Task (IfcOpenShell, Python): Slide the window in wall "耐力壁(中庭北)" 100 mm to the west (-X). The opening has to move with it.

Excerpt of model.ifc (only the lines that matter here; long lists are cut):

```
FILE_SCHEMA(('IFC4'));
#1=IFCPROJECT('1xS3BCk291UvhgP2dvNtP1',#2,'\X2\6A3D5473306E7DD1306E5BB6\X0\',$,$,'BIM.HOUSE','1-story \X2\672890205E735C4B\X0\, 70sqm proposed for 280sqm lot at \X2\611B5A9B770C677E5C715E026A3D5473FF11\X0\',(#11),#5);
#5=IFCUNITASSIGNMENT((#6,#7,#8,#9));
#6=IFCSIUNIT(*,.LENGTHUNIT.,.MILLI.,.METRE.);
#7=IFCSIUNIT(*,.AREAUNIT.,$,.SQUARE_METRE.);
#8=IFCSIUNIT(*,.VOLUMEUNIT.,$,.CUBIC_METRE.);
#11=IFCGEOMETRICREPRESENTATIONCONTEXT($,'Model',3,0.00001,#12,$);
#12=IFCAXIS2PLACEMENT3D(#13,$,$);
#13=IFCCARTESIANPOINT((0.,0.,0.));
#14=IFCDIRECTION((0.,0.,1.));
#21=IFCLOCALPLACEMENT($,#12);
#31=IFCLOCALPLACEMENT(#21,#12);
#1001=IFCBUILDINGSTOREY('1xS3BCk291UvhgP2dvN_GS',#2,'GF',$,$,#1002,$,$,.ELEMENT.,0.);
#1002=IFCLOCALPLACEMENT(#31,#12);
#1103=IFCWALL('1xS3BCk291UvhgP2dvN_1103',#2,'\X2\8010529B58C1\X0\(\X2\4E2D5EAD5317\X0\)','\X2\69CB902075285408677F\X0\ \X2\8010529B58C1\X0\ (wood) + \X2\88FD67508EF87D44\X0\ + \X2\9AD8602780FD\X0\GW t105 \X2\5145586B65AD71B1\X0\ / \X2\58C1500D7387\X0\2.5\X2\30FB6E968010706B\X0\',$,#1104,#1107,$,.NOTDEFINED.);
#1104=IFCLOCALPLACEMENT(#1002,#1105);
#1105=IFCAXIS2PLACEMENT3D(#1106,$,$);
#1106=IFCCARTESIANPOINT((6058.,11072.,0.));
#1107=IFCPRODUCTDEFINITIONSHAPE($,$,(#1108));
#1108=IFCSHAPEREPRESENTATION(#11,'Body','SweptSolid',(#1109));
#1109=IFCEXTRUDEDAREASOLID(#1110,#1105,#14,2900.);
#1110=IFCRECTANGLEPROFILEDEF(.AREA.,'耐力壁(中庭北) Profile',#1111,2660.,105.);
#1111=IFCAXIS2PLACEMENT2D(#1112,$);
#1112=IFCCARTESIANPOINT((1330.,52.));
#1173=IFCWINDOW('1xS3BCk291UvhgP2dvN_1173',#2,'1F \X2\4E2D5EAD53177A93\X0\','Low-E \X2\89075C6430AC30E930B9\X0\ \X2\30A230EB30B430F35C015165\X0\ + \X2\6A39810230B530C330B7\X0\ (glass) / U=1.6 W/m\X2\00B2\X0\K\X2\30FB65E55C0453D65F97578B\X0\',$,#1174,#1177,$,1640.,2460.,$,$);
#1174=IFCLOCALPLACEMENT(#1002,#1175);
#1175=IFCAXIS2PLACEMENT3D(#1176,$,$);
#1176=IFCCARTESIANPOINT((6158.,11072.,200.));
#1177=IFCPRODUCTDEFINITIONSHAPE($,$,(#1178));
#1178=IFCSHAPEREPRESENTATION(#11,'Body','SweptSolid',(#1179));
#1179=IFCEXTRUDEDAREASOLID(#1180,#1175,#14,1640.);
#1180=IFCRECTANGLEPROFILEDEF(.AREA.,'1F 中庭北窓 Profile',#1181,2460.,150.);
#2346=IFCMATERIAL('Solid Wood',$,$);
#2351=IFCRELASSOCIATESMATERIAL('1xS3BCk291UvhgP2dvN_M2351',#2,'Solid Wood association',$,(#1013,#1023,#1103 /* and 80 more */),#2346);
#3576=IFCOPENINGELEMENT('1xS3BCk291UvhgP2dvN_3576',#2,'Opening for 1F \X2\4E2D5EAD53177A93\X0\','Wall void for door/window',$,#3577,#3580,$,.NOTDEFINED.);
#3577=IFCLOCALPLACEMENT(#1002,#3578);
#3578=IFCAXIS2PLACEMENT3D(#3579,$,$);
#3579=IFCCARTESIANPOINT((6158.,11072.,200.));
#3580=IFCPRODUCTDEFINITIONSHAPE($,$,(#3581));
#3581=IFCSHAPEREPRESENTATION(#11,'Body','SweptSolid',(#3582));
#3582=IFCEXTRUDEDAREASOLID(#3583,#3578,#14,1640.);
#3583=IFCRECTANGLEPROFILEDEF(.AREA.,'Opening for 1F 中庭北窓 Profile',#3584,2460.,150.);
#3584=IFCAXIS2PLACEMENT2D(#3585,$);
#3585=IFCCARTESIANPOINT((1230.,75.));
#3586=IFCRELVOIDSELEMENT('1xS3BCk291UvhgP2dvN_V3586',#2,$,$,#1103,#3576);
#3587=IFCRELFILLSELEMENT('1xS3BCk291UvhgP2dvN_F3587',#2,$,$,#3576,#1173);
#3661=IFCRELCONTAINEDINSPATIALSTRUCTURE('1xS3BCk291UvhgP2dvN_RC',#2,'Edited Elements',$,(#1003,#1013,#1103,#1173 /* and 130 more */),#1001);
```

```python
import ifcopenshell
import ifcopenshell.api.geometry
import ifcopenshell.util.placement
import ifcopenshell.util.unit

model = ifcopenshell.open("model.ifc")
unit_scale = ifcopenshell.util.unit.calculate_unit_scale(model)

window = model.by_id(1173)
opening = window.FillsVoids[0].RelatingOpeningElement
wall = opening.VoidsElements[0].RelatingBuildingElement

wall_matrix = ifcopenshell.util.placement.get_local_placement(wall.ObjectPlacement)
shift = wall_matrix[:3, 0] * -0.1 / unit_scale
before = ifcopenshell.util.placement.get_local_placement(window.ObjectPlacement)[:3, 3].copy()

# The window is not placed relative to its opening, so move both.
for product in (opening, window):
    matrix = ifcopenshell.util.placement.get_local_placement(product.ObjectPlacement)
    matrix[:3, 3] += shift
    ifcopenshell.api.geometry.edit_object_placement(model, product=product, matrix=matrix, is_si=False)

after = ifcopenshell.util.placement.get_local_placement(window.ObjectPlacement)[:3, 3]
print("window moved by", (after - before).round(3) + 0.0)

model.write("model_edited.ifc")
```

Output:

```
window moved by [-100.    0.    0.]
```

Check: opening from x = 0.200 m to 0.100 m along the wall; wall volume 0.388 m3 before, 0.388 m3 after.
